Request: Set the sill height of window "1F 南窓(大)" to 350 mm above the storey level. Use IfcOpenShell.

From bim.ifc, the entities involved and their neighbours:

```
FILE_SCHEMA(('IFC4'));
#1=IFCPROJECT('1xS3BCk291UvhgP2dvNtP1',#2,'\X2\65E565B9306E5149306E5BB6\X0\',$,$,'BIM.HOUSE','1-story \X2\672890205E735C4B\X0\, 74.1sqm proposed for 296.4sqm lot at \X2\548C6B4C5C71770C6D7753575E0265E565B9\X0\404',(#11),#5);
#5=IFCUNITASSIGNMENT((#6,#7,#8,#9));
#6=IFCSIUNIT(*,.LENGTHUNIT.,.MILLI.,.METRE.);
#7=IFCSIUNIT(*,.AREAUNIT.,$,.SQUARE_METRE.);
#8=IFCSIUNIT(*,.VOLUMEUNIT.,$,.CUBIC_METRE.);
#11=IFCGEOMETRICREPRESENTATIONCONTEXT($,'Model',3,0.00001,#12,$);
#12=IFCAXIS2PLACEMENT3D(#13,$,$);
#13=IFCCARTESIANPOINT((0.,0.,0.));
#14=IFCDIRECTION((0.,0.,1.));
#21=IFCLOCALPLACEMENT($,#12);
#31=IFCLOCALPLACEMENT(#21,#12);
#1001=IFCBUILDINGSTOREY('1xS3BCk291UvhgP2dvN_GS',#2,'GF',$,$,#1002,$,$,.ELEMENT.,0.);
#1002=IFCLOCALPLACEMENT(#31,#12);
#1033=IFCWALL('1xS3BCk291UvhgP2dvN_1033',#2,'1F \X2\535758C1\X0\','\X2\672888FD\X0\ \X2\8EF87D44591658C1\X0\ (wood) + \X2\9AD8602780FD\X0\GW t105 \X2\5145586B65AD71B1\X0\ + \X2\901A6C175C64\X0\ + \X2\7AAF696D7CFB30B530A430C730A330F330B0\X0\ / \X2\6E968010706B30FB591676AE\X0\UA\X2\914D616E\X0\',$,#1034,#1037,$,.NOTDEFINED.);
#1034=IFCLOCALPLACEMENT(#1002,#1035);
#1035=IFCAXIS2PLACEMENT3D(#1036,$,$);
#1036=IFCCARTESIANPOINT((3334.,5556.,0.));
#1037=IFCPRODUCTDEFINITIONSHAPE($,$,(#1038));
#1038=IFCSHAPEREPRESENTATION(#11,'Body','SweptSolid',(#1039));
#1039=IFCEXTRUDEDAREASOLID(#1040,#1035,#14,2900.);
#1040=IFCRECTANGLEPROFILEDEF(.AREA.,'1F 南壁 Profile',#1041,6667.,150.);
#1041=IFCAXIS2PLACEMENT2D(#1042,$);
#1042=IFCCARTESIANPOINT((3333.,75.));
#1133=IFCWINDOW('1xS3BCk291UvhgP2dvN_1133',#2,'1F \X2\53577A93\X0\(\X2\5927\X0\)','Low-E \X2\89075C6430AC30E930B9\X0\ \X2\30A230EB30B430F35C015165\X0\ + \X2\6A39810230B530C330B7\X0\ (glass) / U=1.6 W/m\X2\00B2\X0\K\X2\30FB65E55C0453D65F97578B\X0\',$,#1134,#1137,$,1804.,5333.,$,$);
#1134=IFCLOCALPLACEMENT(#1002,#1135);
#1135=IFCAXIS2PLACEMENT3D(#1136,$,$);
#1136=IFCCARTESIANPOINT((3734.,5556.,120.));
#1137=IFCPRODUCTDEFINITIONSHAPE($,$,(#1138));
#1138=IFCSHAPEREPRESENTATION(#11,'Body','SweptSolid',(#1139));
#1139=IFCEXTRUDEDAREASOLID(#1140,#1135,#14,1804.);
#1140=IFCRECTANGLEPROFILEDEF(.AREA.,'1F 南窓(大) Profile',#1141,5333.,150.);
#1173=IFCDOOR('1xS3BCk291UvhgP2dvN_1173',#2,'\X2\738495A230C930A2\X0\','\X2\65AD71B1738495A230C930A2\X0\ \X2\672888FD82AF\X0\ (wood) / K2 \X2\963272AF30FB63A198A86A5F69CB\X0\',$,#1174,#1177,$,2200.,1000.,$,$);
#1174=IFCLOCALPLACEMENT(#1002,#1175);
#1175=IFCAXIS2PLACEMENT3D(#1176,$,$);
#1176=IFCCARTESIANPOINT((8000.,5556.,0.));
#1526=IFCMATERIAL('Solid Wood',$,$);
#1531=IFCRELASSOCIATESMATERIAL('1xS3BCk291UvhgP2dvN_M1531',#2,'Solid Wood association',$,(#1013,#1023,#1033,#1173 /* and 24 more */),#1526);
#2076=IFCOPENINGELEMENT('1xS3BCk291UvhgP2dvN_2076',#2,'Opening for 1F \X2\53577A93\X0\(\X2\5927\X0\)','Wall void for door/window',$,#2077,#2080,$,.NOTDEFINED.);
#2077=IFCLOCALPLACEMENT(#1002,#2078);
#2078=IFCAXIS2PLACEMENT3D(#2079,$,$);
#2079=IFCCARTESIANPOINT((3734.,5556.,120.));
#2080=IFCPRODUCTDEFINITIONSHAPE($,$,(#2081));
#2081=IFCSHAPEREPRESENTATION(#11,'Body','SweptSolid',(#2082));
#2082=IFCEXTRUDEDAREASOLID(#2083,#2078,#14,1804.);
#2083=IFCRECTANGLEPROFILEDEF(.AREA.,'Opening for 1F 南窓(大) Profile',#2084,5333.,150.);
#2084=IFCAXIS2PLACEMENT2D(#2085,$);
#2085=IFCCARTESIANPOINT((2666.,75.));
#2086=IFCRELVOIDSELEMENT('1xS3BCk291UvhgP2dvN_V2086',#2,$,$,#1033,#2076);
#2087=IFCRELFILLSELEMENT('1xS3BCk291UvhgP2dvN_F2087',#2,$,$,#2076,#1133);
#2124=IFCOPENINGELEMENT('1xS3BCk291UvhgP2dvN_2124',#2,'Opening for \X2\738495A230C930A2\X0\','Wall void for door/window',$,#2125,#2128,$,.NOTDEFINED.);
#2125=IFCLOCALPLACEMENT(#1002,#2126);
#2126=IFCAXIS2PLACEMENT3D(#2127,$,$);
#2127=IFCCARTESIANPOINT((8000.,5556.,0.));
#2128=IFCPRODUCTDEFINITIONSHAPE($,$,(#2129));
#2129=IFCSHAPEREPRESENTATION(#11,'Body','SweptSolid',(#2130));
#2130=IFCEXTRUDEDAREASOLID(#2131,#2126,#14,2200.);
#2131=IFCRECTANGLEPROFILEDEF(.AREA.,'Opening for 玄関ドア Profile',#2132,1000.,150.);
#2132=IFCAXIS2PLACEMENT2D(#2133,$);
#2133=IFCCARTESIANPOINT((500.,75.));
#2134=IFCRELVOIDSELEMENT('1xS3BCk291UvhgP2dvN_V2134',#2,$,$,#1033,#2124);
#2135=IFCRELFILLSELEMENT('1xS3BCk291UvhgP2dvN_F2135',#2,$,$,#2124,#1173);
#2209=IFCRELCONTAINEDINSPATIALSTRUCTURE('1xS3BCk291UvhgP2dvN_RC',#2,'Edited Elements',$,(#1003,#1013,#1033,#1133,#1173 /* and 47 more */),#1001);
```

```python
import numpy as np
import ifcopenshell
import ifcopenshell.api.geometry
import ifcopenshell.geom
import ifcopenshell.util.element
import ifcopenshell.util.placement
import ifcopenshell.util.shape
import ifcopenshell.util.unit

model = ifcopenshell.open("bim.ifc")
unit_scale = ifcopenshell.util.unit.calculate_unit_scale(model)

window = model.by_guid("1xS3BCk291UvhgP2dvN_1133")
opening = window.FillsVoids[0].RelatingOpeningElement
storey = ifcopenshell.util.element.get_container(window, ifc_class="IfcBuildingStorey")
level = ifcopenshell.util.placement.get_local_placement(storey.ObjectPlacement)[2, 3]

# The opening's origin need not be at the sill, so measure its lowest point.
shape = ifcopenshell.geom.create_shape(ifcopenshell.geom.settings(), opening)
bottom = ifcopenshell.util.shape.get_shape_bottom_elevation(shape, shape.geometry) / unit_scale
dz = level + 0.35 / unit_scale - bottom

shift = np.array([0.0, 0.0, dz])
# The window is not placed relative to its opening, so move both.
for product in (opening, window):
    matrix = ifcopenshell.util.placement.get_local_placement(product.ObjectPlacement)
    matrix[:3, 3] += shift
    ifcopenshell.api.geometry.edit_object_placement(model, product=product, matrix=matrix, is_si=False)

print(f"moved by {dz * unit_scale:+.3f} m")

model.write("bim_edited.ifc")
```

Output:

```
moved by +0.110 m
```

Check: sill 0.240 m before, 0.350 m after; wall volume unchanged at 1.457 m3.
